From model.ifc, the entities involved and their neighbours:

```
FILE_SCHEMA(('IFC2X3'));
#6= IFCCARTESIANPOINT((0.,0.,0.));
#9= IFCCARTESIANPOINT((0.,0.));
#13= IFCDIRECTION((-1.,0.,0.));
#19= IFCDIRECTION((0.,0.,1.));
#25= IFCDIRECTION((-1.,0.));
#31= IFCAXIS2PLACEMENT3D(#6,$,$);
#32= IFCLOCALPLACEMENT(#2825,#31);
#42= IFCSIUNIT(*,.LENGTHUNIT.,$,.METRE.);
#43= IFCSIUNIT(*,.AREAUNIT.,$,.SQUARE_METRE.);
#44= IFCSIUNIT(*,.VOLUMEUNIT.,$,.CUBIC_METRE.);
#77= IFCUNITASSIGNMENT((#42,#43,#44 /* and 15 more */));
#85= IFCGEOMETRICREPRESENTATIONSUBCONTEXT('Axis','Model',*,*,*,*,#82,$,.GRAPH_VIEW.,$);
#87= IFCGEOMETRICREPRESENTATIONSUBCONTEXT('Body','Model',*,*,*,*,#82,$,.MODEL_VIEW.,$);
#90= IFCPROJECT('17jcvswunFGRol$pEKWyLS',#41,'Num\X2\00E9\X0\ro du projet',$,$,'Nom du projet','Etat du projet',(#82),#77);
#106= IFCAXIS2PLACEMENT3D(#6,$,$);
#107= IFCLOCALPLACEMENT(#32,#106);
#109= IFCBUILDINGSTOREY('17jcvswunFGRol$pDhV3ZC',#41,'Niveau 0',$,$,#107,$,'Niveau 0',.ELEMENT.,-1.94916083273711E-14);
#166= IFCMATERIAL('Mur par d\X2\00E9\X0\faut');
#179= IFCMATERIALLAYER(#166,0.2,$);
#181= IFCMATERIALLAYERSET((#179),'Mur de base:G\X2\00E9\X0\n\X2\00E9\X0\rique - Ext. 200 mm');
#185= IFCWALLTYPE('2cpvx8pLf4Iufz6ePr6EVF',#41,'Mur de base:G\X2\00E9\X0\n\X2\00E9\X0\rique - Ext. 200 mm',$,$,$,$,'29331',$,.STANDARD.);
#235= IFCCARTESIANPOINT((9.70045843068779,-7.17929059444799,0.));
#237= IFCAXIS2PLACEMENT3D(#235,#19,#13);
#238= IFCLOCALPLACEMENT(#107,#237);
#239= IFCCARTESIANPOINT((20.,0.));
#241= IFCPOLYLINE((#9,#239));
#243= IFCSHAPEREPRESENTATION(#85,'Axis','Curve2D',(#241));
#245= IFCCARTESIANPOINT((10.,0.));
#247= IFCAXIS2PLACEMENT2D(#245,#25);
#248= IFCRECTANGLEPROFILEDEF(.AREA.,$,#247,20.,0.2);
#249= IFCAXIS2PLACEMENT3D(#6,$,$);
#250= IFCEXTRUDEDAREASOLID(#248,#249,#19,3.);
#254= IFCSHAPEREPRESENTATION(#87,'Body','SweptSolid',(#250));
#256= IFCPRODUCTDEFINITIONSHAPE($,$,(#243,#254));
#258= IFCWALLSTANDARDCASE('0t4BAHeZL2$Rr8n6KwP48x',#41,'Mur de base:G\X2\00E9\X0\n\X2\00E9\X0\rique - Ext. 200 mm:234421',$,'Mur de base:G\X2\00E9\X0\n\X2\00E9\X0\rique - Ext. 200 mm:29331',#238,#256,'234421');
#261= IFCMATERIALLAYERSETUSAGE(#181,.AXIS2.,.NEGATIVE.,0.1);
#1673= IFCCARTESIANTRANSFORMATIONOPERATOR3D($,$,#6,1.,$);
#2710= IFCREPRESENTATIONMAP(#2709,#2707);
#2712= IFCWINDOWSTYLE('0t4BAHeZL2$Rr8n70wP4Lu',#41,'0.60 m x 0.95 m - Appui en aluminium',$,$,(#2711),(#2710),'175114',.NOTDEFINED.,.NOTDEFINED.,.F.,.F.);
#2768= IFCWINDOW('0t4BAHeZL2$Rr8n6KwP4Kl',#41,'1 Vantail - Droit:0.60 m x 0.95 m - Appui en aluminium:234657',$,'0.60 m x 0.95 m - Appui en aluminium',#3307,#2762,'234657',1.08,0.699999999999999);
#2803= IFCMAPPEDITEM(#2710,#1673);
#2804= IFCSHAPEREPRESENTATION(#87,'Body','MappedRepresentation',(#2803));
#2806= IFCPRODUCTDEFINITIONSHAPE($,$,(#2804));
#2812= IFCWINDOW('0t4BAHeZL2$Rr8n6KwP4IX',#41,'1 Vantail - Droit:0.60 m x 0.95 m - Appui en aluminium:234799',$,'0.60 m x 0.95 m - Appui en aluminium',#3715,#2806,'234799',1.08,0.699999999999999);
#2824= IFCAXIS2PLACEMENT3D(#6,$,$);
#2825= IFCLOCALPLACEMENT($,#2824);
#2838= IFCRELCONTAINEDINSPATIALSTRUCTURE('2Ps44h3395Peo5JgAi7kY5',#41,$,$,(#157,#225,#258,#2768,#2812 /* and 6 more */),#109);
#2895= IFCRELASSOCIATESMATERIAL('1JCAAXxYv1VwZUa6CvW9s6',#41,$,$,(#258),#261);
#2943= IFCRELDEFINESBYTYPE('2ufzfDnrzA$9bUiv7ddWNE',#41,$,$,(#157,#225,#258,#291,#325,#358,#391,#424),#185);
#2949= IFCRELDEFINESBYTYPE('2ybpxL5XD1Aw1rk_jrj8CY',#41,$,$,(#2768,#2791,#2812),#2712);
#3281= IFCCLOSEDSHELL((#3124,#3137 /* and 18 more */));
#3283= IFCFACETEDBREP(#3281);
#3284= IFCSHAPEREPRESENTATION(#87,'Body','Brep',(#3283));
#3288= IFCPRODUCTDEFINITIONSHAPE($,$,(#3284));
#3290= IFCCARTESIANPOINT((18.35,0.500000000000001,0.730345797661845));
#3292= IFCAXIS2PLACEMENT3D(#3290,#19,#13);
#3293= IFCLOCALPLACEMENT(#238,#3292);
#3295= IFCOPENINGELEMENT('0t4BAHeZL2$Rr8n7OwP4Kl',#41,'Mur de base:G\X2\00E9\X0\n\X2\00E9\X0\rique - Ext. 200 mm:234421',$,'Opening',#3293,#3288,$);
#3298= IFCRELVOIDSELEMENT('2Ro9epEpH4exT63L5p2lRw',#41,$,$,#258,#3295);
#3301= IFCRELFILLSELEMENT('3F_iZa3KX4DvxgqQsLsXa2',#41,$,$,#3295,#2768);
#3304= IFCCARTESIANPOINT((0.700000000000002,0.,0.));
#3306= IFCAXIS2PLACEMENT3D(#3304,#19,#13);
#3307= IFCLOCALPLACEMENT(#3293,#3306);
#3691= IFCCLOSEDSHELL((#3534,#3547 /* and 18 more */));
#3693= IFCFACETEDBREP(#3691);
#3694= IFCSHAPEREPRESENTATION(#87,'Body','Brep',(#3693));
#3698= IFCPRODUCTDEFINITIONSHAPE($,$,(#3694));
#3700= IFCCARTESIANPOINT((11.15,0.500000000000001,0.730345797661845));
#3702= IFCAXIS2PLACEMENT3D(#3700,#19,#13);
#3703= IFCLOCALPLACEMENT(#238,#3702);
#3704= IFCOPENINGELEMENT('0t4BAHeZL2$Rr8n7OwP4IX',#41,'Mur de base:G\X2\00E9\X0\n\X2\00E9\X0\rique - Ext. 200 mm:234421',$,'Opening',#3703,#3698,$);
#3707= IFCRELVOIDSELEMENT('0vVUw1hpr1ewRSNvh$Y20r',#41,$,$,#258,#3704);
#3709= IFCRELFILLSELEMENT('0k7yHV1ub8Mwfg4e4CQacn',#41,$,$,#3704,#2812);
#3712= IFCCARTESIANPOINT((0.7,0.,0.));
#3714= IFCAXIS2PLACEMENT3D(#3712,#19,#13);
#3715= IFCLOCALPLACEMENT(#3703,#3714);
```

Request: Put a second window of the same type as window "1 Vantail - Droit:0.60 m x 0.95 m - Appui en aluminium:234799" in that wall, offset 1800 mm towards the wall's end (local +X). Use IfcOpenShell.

```python
import ifcopenshell
import ifcopenshell.api.feature
import ifcopenshell.api.geometry
import ifcopenshell.api.root
import ifcopenshell.geom
import ifcopenshell.util.element
import ifcopenshell.util.placement
import ifcopenshell.util.shape

model = ifcopenshell.open("model.ifc")
settings = ifcopenshell.geom.settings()


def volume(element):
    """Net volume in cubic metres, openings subtracted."""
    shape = ifcopenshell.geom.create_shape(settings, element)
    return ifcopenshell.util.shape.get_volume(shape.geometry)


def reuse_history(source, copy):
    """copy_class also copies each property set's owner history, people and application; keep the originals."""
    for rel in copy.IsDefinedBy:
        if rel.is_a("IfcRelDefinesByProperties") and (history := rel.RelatingPropertyDefinition.OwnerHistory):
            rel.RelatingPropertyDefinition.OwnerHistory = source.OwnerHistory
            ifcopenshell.util.element.remove_deep2(model, history)


window = model.by_guid("0t4BAHeZL2$Rr8n6KwP4IX")
opening = window.FillsVoids[0].RelatingOpeningElement
wall = opening.VoidsElements[0].RelatingBuildingElement
before = volume(wall)
shift = ifcopenshell.util.placement.get_local_placement(wall.ObjectPlacement)[:3, 0] * 1.8

# copy_class copies the void relationship, type, container and properties, but no geometry.
new_opening = ifcopenshell.api.root.copy_class(model, product=opening)
new_opening.Representation = ifcopenshell.util.element.copy_deep(
    model, opening.Representation, exclude=["IfcGeometricRepresentationContext", "IfcRepresentationMap"]
)
new_opening.Name = "Mur de base:Générique - Ext. 200 mm"
new_window = ifcopenshell.api.root.copy_class(model, product=window)
new_window.Representation = ifcopenshell.util.element.copy_deep(
    model, window.Representation, exclude=["IfcGeometricRepresentationContext", "IfcRepresentationMap"]
)
new_window.Name = "1 Vantail - Droit:0.60 m x 0.95 m - Appui en aluminium"
new_window.Tag = None
reuse_history(window, new_window)
fills = ifcopenshell.api.feature.add_filling(model, opening=new_opening, element=new_window)
fills.OwnerHistory = new_window.OwnerHistory  # required in IFC2X3

for old, new in ((opening, new_opening), (window, new_window)):
    matrix = ifcopenshell.util.placement.get_local_placement(old.ObjectPlacement)
    matrix[:3, 3] += shift
    ifcopenshell.api.geometry.edit_object_placement(model, product=new, matrix=matrix, is_si=False)

after = volume(wall)

print(f"wall volume {before:.3f} -> {after:.3f} m3")

model.write("model_v2.ifc")
```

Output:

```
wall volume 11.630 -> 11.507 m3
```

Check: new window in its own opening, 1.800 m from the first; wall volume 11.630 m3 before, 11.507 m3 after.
